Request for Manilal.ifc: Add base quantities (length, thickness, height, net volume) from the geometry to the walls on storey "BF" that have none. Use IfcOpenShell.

First a look at what the model holds.

```python
import ifcopenshell
import ifcopenshell.util.element
import ifcopenshell.util.unit

model = ifcopenshell.open("Manilal.ifc")
print(model.schema)
for unit_type in ("LENGTHUNIT", "AREAUNIT", "VOLUMEUNIT"):
    print(unit_type, ifcopenshell.util.unit.calculate_unit_scale(model, unit_type))
storey = next(s for s in model.by_type("IfcBuildingStorey") if s.Name == "BF")
walls = [e for e in ifcopenshell.util.element.get_decomposition(storey) if e.is_a("IfcWall")]
for e in sorted(walls, key=lambda e: e.id()):
    print(e.id(), e.is_a(), e.Name, list(ifcopenshell.util.element.get_psets(e, qtos_only=True)), sep=" | ")
```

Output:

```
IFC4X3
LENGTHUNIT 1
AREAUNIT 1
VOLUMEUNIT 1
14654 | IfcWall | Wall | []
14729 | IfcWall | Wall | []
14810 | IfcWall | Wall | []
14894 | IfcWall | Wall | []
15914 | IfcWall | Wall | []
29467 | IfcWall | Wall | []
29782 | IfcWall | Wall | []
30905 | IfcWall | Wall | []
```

```python
import ifcopenshell
import ifcopenshell.api.pset
import ifcopenshell.geom
import ifcopenshell.util.element
import ifcopenshell.util.shape
import ifcopenshell.util.unit

model = ifcopenshell.open("Manilal.ifc")
unit_scale = ifcopenshell.util.unit.calculate_unit_scale(model)
volume_scale = ifcopenshell.util.unit.calculate_unit_scale(model, "VOLUMEUNIT")
settings = ifcopenshell.geom.settings()

storey = next(s for s in model.by_type("IfcBuildingStorey") if s.Name == "BF")
walls = [e for e in ifcopenshell.util.element.get_decomposition(storey) if e.is_a("IfcWall")]

for e in sorted(walls, key=lambda e: e.id()):
    if ifcopenshell.util.element.get_psets(e, qtos_only=True, should_inherit=False):
        continue
    # Geometry comes back in metres, in the element's own axes.
    shape = ifcopenshell.geom.create_shape(settings, e)
    values = {
        "Length": ifcopenshell.util.shape.get_x(shape.geometry) / unit_scale,
        "Width": ifcopenshell.util.shape.get_y(shape.geometry) / unit_scale,
        "Height": ifcopenshell.util.shape.get_z(shape.geometry) / unit_scale,
        "NetVolume": ifcopenshell.util.shape.get_volume(shape.geometry) / volume_scale,
    }
    qto = ifcopenshell.api.pset.add_qto(model, product=e, name="Qto_WallBaseQuantities")
    ifcopenshell.api.pset.edit_qto(model, qto=qto, properties=values)
    print(e.id(), {k: round(v, 3) for k, v in values.items()})

model.write("Manilal_updated.ifc")
```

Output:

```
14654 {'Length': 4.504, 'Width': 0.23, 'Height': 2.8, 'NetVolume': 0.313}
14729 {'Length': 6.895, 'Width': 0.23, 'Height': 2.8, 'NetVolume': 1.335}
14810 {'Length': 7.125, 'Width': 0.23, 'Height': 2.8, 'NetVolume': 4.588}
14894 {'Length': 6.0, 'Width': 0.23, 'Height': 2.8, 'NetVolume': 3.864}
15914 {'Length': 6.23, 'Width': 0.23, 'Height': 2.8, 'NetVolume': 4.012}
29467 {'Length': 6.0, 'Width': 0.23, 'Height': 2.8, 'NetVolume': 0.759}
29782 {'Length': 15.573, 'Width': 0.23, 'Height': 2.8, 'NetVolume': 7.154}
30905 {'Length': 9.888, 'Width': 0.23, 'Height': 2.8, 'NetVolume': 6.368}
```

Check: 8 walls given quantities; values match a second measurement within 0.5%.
